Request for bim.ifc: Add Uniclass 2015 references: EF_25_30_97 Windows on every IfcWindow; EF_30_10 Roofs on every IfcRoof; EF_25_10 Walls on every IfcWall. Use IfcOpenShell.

First a look at what the model holds.

```python
import ifcopenshell

model = ifcopenshell.open("bim.ifc")
print(model.schema)
print("classifications:", [c.Name for c in model.by_type("IfcClassification")])
for ifc_class in ("IfcDoor", "IfcRoof", "IfcStair", "IfcWall", "IfcWindow"):
    print(ifc_class, len(model.by_type(ifc_class)))
```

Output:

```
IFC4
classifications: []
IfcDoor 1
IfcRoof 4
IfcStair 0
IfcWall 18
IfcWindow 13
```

```python
import ifcopenshell
import ifcopenshell.api.classification

model = ifcopenshell.open("bim.ifc")

system = ifcopenshell.api.classification.add_classification(model, classification="Uniclass 2015")

codes = {
    "IfcWindow": ("EF_25_30_97", "Windows"),
    "IfcRoof": ("EF_30_10", "Roofs"),
    "IfcWall": ("EF_25_10", "Walls"),
}
for ifc_class, (code, name) in codes.items():
    products = model.by_type(ifc_class)
    ifcopenshell.api.classification.add_reference(
        model, products=products, classification=system, identification=code, name=name
    )
    print(code, len(products))

model.write("bim_v2.ifc")
```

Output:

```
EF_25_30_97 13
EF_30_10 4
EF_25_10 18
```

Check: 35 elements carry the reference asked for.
